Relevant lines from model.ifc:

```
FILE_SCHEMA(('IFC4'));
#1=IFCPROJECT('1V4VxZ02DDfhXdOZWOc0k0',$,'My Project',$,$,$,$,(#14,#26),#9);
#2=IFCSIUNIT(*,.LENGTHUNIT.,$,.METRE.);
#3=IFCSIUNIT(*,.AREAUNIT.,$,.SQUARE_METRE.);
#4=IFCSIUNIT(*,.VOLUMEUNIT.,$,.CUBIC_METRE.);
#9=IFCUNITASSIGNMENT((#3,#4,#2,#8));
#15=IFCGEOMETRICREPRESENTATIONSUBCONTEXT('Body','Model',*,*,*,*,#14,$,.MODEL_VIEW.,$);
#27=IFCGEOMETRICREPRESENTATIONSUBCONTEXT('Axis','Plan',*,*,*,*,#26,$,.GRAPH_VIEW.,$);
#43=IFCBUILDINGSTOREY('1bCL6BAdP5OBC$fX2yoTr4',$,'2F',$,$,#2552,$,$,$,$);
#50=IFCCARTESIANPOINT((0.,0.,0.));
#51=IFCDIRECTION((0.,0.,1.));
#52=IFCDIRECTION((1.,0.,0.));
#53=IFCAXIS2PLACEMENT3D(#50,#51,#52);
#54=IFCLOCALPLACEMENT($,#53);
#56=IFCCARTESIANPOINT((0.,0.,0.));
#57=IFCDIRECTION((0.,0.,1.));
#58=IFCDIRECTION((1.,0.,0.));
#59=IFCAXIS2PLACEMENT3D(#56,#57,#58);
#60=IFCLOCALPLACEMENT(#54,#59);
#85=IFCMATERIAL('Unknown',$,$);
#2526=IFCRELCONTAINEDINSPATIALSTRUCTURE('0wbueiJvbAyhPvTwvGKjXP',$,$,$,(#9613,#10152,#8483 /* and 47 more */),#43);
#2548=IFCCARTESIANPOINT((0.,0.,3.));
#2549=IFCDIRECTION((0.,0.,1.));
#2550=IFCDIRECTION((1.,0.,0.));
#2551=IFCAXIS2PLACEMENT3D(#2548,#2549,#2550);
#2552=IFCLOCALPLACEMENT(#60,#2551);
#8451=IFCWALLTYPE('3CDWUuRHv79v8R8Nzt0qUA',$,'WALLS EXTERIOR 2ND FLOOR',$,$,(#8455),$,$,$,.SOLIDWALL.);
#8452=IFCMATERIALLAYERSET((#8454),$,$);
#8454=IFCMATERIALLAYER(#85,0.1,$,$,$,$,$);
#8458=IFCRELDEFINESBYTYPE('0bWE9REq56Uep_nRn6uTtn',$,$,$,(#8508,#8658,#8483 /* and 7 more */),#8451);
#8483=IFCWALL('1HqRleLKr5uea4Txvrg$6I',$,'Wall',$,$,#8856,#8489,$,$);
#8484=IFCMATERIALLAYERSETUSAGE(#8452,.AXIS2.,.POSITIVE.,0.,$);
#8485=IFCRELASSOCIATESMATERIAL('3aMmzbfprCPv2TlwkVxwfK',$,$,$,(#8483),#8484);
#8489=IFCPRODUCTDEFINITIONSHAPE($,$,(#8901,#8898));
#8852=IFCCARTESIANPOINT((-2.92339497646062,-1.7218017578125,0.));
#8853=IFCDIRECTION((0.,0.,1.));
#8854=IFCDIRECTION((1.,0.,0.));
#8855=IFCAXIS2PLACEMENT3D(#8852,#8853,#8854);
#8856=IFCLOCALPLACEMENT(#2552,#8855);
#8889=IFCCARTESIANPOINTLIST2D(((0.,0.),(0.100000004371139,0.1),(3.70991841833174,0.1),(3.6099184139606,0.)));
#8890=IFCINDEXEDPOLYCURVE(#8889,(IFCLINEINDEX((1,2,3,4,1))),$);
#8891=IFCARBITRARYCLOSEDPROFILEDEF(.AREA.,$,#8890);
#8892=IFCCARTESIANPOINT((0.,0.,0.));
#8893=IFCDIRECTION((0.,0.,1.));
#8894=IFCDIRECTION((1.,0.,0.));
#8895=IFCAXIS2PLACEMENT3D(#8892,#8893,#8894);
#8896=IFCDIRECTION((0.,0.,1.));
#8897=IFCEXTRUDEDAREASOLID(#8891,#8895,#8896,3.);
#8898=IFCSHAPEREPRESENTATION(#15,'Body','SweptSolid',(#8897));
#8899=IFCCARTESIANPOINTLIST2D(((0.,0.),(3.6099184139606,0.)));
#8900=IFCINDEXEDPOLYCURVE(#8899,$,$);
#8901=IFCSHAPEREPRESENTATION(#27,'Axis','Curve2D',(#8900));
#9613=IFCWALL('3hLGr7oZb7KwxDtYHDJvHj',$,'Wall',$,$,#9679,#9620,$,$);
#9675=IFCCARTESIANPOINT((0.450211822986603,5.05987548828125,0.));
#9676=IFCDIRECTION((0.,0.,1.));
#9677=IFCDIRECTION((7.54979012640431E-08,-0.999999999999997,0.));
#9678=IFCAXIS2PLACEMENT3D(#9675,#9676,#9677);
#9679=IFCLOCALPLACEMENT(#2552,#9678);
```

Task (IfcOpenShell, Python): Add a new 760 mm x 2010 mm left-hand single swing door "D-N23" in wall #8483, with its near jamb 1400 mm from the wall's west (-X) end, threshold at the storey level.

```python
import numpy as np
import ifcopenshell
import ifcopenshell.api.feature
import ifcopenshell.api.geometry
import ifcopenshell.api.root
import ifcopenshell.api.spatial
import ifcopenshell.geom
import ifcopenshell.util.element
import ifcopenshell.util.placement
import ifcopenshell.util.representation
import ifcopenshell.util.shape
import ifcopenshell.util.unit

model = ifcopenshell.open("model.ifc")
unit_scale = ifcopenshell.util.unit.calculate_unit_scale(model)
settings = ifcopenshell.geom.settings()


def volume(element):
    """Net volume in cubic metres, openings subtracted."""
    shape = ifcopenshell.geom.create_shape(settings, element)
    return ifcopenshell.util.shape.get_volume(shape.geometry)


wall = model.by_guid("1HqRleLKr5uea4Txvrg$6I")
storey = ifcopenshell.util.element.get_container(wall, ifc_class="IfcBuildingStorey")
context = ifcopenshell.util.representation.get_context(model, "Model", "Body", "MODEL_VIEW")
before = volume(wall)

width, height, from_end, sill = 0.76, 2.01, 1.4, 0.0  # metres

# The wall runs along its own X axis, and the end named is its -X end.
wall_shape = ifcopenshell.geom.create_shape(settings, wall)
x, y, z = ifcopenshell.util.shape.get_vertices(wall_shape.geometry).T
start = x.min() + from_end
face, thickness = float(y.min()), float(y.max() - y.min())
wall_matrix = ifcopenshell.util.placement.get_local_placement(wall.ObjectPlacement)
level = ifcopenshell.util.placement.get_local_placement(storey.ObjectPlacement)[2, 3]


def in_wall(x, y):
    """Placement at x, y metres in the wall's axes, at sill height."""
    matrix = wall_matrix.copy()
    matrix[:, 3] = wall_matrix @ np.array([x / unit_scale, y / unit_scale, 0.0, 1.0])
    matrix[2, 3] = level + sill / unit_scale
    return matrix


# Opening: a box that overshoots both wall faces by 50 mm.
opening = ifcopenshell.api.root.create_entity(model, ifc_class="IfcOpeningElement", predefined_type="OPENING")
box = ifcopenshell.api.geometry.add_wall_representation(
    model, context=context, length=width, height=height, thickness=thickness + 0.1
)
ifcopenshell.api.geometry.assign_representation(model, product=opening, representation=box)
ifcopenshell.api.geometry.edit_object_placement(model, product=opening, matrix=in_wall(start, face - 0.05), is_si=False)
ifcopenshell.api.feature.add_feature(model, feature=opening, element=wall)

door = ifcopenshell.api.root.create_entity(model, ifc_class="IfcDoor", name="D-N23", predefined_type="DOOR")
door.OverallWidth, door.OverallHeight = width / unit_scale, height / unit_scale
door.OperationType = "SINGLE_SWING_LEFT"
body = ifcopenshell.api.geometry.add_door_representation(
    model,
    context=context,
    overall_width=door.OverallWidth,
    overall_height=door.OverallHeight,
    operation_type="SINGLE_SWING_LEFT",
    lining_properties={"LiningDepth": thickness / unit_scale, "ThresholdDepth": thickness / unit_scale},
)
ifcopenshell.api.geometry.assign_representation(model, product=door, representation=body)
ifcopenshell.api.spatial.assign_container(model, products=[door], relating_structure=storey)
ifcopenshell.api.feature.add_filling(model, opening=opening, element=door)

# The lining spans the wall, so the door starts at the wall face.
ifcopenshell.api.geometry.edit_object_placement(model, product=door, matrix=in_wall(start, face), is_si=False)

after = volume(wall)

print(f"wall volume {before:.3f} -> {after:.3f} m3")

model.write("model_rev.ifc")
```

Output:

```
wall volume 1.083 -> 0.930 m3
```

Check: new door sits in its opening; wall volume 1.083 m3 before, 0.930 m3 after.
